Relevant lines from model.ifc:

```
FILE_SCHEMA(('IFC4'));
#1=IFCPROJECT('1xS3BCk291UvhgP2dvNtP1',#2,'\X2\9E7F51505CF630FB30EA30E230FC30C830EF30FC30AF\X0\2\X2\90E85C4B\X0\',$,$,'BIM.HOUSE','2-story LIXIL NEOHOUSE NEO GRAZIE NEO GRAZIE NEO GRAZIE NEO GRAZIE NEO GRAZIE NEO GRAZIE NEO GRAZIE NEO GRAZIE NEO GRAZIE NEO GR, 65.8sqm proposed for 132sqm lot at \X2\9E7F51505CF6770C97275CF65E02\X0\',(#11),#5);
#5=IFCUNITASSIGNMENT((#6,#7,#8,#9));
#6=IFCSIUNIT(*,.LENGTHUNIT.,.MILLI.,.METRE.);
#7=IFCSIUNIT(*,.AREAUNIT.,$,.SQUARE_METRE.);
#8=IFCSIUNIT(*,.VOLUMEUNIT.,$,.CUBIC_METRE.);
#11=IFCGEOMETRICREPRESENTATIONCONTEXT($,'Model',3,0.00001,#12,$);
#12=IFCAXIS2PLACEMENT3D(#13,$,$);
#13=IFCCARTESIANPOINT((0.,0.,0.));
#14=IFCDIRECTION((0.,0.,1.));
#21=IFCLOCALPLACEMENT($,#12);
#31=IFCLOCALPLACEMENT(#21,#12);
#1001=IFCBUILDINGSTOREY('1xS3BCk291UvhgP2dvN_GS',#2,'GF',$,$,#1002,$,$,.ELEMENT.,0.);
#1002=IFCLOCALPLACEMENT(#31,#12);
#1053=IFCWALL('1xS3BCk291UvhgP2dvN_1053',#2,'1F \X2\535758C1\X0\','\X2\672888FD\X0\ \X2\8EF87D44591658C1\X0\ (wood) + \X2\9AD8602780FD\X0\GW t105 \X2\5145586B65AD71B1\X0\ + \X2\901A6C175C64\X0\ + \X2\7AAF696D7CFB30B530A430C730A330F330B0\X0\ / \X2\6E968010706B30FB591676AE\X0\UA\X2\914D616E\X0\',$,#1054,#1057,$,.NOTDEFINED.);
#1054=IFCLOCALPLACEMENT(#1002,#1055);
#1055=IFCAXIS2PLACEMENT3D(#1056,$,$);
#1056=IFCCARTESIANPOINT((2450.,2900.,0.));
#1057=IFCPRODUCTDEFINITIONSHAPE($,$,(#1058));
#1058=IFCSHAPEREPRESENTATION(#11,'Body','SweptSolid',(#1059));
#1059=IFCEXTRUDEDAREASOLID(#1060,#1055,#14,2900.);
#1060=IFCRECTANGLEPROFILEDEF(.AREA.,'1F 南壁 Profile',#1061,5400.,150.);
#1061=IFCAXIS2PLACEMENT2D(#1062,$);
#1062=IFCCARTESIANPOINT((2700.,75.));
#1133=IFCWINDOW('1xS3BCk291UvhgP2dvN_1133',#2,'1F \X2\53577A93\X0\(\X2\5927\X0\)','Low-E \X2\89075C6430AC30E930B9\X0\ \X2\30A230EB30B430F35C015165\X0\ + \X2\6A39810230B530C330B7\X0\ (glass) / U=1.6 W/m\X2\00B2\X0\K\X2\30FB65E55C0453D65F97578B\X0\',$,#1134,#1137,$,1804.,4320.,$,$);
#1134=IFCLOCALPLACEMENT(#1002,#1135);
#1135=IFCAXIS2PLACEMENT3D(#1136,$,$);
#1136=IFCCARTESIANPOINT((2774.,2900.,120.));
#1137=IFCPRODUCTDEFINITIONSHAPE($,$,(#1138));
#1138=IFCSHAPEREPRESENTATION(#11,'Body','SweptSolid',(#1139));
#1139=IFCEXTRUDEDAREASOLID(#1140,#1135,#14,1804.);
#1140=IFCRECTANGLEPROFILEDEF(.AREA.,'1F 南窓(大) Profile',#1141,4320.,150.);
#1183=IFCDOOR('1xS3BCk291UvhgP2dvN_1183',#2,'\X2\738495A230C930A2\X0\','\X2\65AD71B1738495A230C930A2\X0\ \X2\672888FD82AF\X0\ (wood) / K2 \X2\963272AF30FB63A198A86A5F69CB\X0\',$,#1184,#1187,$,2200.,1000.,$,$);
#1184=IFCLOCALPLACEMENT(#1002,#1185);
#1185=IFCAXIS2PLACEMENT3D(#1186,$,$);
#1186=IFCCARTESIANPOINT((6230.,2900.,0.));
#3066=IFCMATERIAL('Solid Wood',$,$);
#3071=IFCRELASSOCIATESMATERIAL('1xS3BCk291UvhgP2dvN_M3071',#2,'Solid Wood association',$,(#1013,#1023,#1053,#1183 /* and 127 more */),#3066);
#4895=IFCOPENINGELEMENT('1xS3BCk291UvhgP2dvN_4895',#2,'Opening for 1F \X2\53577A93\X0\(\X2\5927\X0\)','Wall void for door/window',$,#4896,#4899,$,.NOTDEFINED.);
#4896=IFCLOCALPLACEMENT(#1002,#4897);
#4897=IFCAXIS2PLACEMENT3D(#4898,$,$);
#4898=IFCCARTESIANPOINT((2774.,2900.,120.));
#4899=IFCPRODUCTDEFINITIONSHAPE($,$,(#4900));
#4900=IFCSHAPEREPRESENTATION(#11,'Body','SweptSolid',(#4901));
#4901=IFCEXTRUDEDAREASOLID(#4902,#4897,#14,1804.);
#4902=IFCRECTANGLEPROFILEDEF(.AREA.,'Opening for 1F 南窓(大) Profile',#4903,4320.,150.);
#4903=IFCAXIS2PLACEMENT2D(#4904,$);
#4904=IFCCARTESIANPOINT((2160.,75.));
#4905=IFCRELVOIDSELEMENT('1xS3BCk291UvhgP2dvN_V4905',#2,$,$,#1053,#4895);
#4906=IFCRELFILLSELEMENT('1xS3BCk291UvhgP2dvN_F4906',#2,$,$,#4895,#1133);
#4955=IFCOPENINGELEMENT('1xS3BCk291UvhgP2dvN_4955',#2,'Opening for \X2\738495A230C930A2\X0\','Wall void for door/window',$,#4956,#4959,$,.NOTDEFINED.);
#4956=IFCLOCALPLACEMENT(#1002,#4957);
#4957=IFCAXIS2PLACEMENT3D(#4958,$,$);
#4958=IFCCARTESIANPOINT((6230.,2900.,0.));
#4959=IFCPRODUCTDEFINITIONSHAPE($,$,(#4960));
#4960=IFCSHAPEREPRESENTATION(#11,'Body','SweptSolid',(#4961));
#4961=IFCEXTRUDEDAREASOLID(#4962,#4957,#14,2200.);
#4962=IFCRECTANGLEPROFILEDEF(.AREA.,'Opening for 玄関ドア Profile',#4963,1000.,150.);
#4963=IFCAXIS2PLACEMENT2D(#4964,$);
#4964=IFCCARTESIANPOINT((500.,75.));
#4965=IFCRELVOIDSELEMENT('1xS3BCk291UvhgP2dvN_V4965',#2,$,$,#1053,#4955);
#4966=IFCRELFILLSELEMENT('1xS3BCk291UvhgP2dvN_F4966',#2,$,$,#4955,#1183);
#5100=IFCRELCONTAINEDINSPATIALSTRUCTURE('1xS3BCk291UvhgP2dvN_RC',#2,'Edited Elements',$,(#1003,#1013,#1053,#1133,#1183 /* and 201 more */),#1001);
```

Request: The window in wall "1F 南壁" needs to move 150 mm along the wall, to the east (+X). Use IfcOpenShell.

```python
import ifcopenshell
import ifcopenshell.api.geometry
import ifcopenshell.util.placement
import ifcopenshell.util.unit

model = ifcopenshell.open("model.ifc")
unit_scale = ifcopenshell.util.unit.calculate_unit_scale(model)

window = model.by_guid("1xS3BCk291UvhgP2dvN_1133")
opening = window.FillsVoids[0].RelatingOpeningElement
wall = opening.VoidsElements[0].RelatingBuildingElement

wall_matrix = ifcopenshell.util.placement.get_local_placement(wall.ObjectPlacement)
shift = wall_matrix[:3, 0] * 0.15 / unit_scale
before = ifcopenshell.util.placement.get_local_placement(window.ObjectPlacement)[:3, 3].copy()

# The window is not placed relative to its opening, so move both.
for product in (opening, window):
    matrix = ifcopenshell.util.placement.get_local_placement(product.ObjectPlacement)
    matrix[:3, 3] += shift
    ifcopenshell.api.geometry.edit_object_placement(model, product=product, matrix=matrix, is_si=False)

after = ifcopenshell.util.placement.get_local_placement(window.ObjectPlacement)[:3, 3]
print("window moved by", (after - before).round(3) + 0.0)

model.write("model-out.ifc")
```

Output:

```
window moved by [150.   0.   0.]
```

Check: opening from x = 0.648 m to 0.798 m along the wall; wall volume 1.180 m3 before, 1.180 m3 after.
